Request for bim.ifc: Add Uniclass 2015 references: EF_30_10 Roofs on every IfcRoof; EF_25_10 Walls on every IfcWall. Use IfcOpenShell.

First a look at what the model holds.

```python
import ifcopenshell

model = ifcopenshell.open("bim.ifc")
print(model.schema)
print("classifications:", [c.Name for c in model.by_type("IfcClassification")])
for ifc_class in ("IfcDoor", "IfcRoof", "IfcStair", "IfcWall", "IfcWindow"):
    print(ifc_class, len(model.by_type(ifc_class)))
```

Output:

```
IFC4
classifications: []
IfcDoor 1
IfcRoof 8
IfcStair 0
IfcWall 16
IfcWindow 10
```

```python
import ifcopenshell
import ifcopenshell.api.classification

model = ifcopenshell.open("bim.ifc")

system = ifcopenshell.api.classification.add_classification(model, classification="Uniclass 2015")

codes = {
    "IfcRoof": ("EF_30_10", "Roofs"),
    "IfcWall": ("EF_25_10", "Walls"),
}
for ifc_class, (code, name) in codes.items():
    products = model.by_type(ifc_class)
    ifcopenshell.api.classification.add_reference(
        model, products=products, classification=system, identification=code, name=name
    )
    print(code, len(products))

model.write("bim-out.ifc")
```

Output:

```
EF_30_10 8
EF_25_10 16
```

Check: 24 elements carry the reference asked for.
